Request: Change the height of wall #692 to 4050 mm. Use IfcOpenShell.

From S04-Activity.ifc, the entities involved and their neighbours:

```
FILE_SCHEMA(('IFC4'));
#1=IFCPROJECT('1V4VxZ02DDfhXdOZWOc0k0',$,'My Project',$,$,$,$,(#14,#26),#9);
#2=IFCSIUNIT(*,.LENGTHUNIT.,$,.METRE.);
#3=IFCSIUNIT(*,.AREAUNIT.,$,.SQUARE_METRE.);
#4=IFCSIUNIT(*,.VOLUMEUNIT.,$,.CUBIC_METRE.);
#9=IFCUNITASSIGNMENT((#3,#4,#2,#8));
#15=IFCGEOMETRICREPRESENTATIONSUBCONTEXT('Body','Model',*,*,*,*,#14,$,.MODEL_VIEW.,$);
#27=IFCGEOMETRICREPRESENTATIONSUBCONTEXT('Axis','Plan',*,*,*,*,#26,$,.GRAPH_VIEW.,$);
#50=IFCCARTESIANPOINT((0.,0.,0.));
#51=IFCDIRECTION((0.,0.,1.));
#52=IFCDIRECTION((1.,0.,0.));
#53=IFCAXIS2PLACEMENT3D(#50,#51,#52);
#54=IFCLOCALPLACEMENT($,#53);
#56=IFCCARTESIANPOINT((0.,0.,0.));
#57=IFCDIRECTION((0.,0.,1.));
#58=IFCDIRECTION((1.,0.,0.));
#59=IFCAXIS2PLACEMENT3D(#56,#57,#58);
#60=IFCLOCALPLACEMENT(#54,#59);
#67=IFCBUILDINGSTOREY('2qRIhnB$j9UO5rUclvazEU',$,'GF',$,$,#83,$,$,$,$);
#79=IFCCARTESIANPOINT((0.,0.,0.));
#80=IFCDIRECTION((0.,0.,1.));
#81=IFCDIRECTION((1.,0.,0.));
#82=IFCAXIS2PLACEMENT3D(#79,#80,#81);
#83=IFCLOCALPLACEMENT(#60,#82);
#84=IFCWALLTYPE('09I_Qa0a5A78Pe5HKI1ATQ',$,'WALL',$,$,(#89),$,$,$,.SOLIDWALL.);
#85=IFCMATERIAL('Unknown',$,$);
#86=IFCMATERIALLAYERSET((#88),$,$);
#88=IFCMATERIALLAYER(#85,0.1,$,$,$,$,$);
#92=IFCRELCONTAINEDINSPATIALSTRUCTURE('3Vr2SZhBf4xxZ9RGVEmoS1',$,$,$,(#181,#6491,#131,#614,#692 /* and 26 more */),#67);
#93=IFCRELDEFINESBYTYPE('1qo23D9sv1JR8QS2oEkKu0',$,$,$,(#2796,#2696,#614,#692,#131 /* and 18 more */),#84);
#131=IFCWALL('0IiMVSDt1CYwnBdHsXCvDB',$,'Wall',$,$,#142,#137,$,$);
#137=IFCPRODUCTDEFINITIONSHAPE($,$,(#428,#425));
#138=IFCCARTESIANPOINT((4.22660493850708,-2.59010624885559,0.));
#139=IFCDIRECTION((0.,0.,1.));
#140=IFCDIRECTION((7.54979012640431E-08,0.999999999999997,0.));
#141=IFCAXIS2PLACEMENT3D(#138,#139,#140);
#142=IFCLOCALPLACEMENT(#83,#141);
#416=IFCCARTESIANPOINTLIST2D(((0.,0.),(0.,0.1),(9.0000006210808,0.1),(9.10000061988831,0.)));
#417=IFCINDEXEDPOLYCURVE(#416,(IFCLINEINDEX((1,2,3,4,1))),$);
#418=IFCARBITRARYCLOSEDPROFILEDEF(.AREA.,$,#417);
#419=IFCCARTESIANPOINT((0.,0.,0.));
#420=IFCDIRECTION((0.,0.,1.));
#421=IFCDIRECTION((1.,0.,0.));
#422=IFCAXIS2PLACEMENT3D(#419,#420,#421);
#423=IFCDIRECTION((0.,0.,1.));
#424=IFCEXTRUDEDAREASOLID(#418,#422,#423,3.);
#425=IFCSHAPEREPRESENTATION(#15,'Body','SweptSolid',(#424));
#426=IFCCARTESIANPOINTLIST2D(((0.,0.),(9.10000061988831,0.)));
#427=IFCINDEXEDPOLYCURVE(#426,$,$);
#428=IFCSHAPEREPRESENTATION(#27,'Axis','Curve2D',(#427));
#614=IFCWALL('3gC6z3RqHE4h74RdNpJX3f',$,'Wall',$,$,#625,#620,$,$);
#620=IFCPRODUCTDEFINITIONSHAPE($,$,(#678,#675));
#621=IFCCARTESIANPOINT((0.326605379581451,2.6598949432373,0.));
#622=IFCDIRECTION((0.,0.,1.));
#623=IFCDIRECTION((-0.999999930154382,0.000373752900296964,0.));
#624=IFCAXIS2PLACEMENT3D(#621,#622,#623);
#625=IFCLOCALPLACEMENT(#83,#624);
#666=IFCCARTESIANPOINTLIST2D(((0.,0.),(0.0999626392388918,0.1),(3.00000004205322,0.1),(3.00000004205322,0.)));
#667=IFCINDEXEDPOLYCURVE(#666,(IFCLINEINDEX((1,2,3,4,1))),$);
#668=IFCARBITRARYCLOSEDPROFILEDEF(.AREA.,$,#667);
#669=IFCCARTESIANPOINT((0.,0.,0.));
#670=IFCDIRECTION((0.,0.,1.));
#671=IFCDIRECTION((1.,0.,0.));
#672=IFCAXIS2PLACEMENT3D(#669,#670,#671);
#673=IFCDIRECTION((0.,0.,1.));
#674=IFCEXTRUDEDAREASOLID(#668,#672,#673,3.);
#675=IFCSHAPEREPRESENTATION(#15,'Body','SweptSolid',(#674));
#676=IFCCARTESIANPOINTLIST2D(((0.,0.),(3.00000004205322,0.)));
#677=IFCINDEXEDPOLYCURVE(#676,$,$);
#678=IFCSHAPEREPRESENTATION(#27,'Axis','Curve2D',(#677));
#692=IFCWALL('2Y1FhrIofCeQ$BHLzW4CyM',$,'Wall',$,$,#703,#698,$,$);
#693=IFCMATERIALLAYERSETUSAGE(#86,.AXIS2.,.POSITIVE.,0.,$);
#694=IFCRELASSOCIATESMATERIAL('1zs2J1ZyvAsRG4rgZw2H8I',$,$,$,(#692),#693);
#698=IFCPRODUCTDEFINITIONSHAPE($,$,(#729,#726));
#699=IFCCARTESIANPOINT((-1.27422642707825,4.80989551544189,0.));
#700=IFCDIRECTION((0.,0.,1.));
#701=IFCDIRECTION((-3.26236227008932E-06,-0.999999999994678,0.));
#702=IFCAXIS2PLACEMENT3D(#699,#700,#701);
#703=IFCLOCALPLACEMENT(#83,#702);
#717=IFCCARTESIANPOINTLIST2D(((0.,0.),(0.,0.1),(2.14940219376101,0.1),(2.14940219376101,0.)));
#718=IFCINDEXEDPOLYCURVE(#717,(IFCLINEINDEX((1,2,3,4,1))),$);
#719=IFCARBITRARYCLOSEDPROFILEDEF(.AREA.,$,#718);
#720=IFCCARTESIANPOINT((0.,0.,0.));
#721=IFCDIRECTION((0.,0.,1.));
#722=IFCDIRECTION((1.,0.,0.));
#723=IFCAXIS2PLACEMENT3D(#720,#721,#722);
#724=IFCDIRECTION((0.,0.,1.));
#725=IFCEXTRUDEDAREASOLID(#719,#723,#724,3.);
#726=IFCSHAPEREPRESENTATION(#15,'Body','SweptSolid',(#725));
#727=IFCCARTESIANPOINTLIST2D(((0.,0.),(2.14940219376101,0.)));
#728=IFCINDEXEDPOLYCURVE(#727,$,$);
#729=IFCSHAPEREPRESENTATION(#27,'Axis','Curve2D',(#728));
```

```python
import ifcopenshell
import ifcopenshell.geom
import ifcopenshell.util.representation
import ifcopenshell.util.shape

model = ifcopenshell.open("S04-Activity.ifc")
settings = ifcopenshell.geom.settings()


def volume(element):
    """Net volume in cubic metres, openings subtracted."""
    shape = ifcopenshell.geom.create_shape(settings, element)
    return ifcopenshell.util.shape.get_volume(shape.geometry)


wall = model.by_guid("2Y1FhrIofCeQ$BHLzW4CyM")
before = volume(wall)

body = ifcopenshell.util.representation.get_representation(wall, "Model", "Body")
solid = body.Items[0]
old_height = solid.Depth
solid.Depth = 4.05
after = volume(wall)

print(f"height {old_height:g} -> {solid.Depth:g}, volume {before:.3f} -> {after:.3f} m3")

model.write("S04-Activity_v2.ifc")
```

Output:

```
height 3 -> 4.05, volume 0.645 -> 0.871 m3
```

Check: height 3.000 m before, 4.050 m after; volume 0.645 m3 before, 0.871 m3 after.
